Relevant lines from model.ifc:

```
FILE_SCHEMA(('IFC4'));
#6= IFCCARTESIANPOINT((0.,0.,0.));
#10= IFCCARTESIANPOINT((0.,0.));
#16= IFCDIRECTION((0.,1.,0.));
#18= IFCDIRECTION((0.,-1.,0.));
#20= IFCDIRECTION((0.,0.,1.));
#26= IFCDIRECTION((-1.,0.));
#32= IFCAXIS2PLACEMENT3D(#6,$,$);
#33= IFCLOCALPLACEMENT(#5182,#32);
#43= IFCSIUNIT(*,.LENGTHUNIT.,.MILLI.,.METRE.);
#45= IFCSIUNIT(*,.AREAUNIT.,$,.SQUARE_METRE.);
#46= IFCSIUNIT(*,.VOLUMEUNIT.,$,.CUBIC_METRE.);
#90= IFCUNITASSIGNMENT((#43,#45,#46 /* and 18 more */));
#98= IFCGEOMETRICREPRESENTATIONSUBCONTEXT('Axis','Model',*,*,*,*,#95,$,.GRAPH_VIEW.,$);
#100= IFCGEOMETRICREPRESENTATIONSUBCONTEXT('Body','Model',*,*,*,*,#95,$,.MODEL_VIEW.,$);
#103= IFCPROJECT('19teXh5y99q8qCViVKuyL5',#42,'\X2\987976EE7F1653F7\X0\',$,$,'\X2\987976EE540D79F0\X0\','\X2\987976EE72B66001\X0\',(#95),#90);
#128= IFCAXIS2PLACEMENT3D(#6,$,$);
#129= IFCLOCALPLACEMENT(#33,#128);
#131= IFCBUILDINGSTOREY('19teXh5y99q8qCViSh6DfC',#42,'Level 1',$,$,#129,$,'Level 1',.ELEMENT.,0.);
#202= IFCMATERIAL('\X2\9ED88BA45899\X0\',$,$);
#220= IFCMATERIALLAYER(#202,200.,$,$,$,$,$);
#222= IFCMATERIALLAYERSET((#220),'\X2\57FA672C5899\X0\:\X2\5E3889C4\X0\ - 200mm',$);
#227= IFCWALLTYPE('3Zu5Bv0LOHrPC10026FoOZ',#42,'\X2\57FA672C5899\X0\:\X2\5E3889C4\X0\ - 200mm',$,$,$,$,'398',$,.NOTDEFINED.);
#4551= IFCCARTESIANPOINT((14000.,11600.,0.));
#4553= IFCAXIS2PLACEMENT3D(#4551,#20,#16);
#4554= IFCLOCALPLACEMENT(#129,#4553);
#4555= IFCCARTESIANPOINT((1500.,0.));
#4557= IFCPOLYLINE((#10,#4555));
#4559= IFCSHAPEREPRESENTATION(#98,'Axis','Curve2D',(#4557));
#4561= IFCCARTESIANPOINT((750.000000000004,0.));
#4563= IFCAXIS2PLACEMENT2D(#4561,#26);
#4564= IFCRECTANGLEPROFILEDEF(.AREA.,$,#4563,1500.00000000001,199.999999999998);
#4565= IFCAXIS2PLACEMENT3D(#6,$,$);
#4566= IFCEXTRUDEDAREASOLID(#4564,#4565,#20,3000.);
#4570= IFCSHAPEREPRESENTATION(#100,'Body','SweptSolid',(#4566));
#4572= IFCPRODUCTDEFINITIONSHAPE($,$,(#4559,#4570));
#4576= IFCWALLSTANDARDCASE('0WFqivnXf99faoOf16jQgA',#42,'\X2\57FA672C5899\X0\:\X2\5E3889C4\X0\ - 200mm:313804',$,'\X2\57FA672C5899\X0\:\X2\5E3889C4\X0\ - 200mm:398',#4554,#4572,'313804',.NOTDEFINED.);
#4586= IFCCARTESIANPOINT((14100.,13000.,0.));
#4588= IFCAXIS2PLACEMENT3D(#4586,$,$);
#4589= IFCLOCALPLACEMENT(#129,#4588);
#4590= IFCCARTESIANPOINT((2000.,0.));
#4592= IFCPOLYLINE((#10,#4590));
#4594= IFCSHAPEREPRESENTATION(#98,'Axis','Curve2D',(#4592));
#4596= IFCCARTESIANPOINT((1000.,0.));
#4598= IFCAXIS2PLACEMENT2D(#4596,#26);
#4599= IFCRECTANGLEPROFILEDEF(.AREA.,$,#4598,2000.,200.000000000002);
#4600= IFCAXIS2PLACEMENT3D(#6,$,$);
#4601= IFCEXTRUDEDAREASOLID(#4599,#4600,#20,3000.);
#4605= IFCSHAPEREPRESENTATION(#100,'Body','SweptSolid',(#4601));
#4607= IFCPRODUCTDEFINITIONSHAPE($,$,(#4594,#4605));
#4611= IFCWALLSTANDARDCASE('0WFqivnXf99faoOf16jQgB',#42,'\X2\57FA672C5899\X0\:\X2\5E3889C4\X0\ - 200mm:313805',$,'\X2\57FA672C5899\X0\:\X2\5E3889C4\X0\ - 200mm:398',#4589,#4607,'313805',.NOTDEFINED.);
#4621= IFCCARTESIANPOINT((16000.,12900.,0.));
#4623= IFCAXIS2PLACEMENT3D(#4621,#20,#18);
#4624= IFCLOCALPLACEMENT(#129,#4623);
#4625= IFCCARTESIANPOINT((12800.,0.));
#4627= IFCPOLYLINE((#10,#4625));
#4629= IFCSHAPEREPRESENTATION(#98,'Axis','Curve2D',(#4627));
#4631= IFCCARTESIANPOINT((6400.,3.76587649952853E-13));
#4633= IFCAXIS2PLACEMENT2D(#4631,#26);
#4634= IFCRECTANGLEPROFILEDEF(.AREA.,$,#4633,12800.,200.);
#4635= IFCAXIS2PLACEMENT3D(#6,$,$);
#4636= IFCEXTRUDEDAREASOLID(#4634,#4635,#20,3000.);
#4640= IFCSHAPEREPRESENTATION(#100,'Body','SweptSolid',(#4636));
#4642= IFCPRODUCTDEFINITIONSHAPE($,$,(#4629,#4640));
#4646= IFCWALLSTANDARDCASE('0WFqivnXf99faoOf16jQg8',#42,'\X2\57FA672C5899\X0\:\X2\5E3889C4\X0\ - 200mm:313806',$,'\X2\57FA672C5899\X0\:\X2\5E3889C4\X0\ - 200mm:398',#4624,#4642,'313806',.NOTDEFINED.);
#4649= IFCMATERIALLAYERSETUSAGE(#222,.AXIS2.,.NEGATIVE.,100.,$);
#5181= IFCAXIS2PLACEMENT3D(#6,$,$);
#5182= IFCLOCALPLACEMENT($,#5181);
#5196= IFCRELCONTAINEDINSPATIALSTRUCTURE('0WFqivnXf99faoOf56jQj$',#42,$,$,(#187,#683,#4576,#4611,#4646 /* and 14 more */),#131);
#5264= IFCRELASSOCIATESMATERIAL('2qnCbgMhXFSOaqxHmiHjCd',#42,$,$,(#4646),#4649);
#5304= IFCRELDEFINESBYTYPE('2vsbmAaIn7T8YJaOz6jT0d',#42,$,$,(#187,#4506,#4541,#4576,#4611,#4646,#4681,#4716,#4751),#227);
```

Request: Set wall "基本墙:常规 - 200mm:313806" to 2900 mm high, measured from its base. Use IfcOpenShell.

```python
import ifcopenshell
import ifcopenshell.geom
import ifcopenshell.util.representation
import ifcopenshell.util.shape

model = ifcopenshell.open("model.ifc")
settings = ifcopenshell.geom.settings()


def volume(element):
    """Net volume in cubic metres, openings subtracted."""
    shape = ifcopenshell.geom.create_shape(settings, element)
    return ifcopenshell.util.shape.get_volume(shape.geometry)


wall = model.by_guid("0WFqivnXf99faoOf16jQg8")
before = volume(wall)

body = ifcopenshell.util.representation.get_representation(wall, "Model", "Body")
solid = body.Items[0]
old_height = solid.Depth
solid.Depth = 2900.0
after = volume(wall)

print(f"height {old_height:g} -> {solid.Depth:g}, volume {before:.3f} -> {after:.3f} m3")

model.write("model_v2.ifc")
```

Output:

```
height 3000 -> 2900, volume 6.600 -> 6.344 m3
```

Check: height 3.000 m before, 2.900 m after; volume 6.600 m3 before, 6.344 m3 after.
